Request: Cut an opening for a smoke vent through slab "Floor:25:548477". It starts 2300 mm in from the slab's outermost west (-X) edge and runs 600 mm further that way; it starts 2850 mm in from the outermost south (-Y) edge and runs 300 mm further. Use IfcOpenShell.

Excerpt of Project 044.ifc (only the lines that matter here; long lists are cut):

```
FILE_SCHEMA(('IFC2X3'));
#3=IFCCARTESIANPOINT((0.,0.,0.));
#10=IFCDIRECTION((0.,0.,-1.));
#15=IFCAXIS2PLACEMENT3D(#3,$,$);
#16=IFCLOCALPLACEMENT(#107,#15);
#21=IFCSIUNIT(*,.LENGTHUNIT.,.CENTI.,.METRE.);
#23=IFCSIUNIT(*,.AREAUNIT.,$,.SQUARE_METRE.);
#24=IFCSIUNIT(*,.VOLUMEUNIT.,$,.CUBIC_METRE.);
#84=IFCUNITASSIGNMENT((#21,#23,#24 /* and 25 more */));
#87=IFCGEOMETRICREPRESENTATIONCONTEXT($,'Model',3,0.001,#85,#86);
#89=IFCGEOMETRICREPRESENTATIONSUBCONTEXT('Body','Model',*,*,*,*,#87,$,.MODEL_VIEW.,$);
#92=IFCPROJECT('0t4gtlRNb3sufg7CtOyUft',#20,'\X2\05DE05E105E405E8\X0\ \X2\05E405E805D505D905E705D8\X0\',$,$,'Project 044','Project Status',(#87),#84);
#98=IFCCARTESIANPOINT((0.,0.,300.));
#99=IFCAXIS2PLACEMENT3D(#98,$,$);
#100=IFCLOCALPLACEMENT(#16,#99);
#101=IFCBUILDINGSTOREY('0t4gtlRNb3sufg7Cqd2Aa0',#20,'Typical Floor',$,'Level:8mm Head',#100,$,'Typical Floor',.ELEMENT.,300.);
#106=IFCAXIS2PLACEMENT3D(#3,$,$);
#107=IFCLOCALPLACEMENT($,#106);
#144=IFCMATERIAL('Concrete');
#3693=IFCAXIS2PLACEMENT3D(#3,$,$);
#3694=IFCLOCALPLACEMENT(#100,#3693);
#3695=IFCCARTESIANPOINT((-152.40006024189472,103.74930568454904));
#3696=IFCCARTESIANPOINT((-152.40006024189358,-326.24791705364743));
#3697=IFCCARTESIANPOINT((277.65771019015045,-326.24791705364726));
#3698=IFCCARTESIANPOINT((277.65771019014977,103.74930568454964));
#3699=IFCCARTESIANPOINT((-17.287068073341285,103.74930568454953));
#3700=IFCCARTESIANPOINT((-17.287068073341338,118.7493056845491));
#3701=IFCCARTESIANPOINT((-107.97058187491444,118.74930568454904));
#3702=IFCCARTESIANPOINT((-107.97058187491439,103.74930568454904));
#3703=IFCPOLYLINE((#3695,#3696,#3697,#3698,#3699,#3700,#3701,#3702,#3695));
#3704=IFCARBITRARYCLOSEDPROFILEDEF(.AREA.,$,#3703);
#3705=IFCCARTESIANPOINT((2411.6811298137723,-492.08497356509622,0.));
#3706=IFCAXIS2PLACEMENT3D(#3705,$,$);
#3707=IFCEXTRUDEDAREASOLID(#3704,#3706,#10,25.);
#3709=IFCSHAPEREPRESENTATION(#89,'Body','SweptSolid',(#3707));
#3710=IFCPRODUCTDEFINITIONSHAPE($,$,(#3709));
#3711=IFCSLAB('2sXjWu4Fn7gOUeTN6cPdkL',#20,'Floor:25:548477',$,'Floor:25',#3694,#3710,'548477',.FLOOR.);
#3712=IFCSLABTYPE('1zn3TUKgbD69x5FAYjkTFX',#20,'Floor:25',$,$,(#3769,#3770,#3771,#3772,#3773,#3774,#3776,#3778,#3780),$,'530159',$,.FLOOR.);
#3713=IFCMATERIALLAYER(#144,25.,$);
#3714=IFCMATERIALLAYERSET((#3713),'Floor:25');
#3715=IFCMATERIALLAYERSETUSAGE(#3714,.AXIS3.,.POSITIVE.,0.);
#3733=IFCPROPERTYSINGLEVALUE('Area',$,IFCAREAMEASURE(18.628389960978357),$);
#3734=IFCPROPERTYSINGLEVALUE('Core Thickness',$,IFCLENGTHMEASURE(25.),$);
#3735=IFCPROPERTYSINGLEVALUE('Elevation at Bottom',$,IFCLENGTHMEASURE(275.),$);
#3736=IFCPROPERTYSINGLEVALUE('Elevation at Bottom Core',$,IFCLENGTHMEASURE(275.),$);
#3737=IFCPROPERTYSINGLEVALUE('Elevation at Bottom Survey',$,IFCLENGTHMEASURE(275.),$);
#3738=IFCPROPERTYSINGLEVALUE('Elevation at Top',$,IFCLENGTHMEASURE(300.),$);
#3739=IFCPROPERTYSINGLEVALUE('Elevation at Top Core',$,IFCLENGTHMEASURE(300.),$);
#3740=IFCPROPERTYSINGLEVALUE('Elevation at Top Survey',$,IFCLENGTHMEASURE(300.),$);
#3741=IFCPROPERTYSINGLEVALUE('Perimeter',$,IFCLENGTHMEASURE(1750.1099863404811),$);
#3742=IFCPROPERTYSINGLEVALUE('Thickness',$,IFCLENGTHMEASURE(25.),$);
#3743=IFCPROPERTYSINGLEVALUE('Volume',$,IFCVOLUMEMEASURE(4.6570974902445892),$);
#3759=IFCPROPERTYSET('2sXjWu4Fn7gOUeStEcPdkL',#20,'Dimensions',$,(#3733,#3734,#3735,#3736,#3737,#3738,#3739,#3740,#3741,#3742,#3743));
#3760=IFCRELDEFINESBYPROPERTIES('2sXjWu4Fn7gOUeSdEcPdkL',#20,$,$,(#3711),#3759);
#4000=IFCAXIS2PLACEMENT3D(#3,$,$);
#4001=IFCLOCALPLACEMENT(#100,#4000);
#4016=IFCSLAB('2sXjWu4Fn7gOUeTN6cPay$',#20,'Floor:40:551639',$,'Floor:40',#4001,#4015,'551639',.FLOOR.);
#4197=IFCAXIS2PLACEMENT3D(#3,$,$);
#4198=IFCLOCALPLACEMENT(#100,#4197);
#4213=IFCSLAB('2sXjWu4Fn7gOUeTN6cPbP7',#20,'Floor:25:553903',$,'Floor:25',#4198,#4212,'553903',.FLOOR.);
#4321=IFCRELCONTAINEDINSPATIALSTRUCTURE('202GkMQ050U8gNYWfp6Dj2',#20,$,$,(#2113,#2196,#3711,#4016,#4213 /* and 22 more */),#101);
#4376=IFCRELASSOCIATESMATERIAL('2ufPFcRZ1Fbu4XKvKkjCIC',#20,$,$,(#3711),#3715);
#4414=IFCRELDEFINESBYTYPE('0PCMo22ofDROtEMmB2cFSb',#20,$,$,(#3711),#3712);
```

```python
import numpy as np
import ifcopenshell
import ifcopenshell.api.feature
import ifcopenshell.api.geometry
import ifcopenshell.api.pset
import ifcopenshell.api.root
import ifcopenshell.geom
import ifcopenshell.util.element
import ifcopenshell.util.placement
import ifcopenshell.util.representation
import ifcopenshell.util.shape
import ifcopenshell.util.unit

model = ifcopenshell.open("Project 044.ifc")
unit_scale = ifcopenshell.util.unit.calculate_unit_scale(model)
area_scale = ifcopenshell.util.unit.calculate_unit_scale(model, "AREAUNIT")
volume_scale = ifcopenshell.util.unit.calculate_unit_scale(model, "VOLUMEUNIT")
settings = ifcopenshell.geom.settings()


def volume(element):
    """Net volume in cubic metres, openings subtracted."""
    shape = ifcopenshell.geom.create_shape(settings, element)
    return ifcopenshell.util.shape.get_volume(shape.geometry)


slab = model.by_id(3711)
before = volume(slab)

# Extent in the slab's own axes, in metres. The edges named are its -X and -Y sides.
slab_shape = ifcopenshell.geom.create_shape(settings, slab)
vertices = ifcopenshell.util.shape.get_vertices(slab_shape.geometry)
x_min, y_min, bottom = vertices.min(axis=0)
top = vertices[:, 2].max()

opening = ifcopenshell.api.root.create_entity(model, ifc_class="IfcOpeningElement", name="Smoke vent opening")
context = ifcopenshell.util.representation.get_context(model, "Model", "Body", "MODEL_VIEW")
width, depth = 0.6, 0.3
outline = [(0.0, 0.0), (width, 0.0), (width, depth), (0.0, depth), (0.0, 0.0)]
# Overshoot both faces by 50 mm so the cut is clean.
shape = ifcopenshell.api.geometry.add_slab_representation(
    model, context=context, depth=top - bottom + 0.1, polyline=outline
)
ifcopenshell.api.geometry.assign_representation(model, product=opening, representation=shape)

matrix = ifcopenshell.util.placement.get_local_placement(slab.ObjectPlacement)
matrix[:, 3] = matrix @ np.append(np.array([x_min + 2.3, y_min + 2.85, bottom - 0.05]) / unit_scale, 1.0)
ifcopenshell.api.geometry.edit_object_placement(model, product=opening, matrix=matrix, is_si=False)
ifcopenshell.api.feature.add_feature(model, feature=opening, element=slab)

after = volume(slab)

# Update the slab's stored quantities.
pset = model.by_id(ifcopenshell.util.element.get_pset(slab, "Dimensions", should_inherit=False)["id"])
ifcopenshell.api.pset.edit_pset(model, pset=pset, properties={
    "Area": model.create_entity("IfcAreaMeasure", after / (top - bottom) / area_scale),
    "Volume": model.create_entity("IfcVolumeMeasure", after / volume_scale),
})

print(f"slab volume {before:.3f} -> {after:.3f} m3")

model.write("Project 044_rev.ifc")
```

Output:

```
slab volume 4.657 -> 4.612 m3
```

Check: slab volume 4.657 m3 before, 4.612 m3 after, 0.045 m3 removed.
